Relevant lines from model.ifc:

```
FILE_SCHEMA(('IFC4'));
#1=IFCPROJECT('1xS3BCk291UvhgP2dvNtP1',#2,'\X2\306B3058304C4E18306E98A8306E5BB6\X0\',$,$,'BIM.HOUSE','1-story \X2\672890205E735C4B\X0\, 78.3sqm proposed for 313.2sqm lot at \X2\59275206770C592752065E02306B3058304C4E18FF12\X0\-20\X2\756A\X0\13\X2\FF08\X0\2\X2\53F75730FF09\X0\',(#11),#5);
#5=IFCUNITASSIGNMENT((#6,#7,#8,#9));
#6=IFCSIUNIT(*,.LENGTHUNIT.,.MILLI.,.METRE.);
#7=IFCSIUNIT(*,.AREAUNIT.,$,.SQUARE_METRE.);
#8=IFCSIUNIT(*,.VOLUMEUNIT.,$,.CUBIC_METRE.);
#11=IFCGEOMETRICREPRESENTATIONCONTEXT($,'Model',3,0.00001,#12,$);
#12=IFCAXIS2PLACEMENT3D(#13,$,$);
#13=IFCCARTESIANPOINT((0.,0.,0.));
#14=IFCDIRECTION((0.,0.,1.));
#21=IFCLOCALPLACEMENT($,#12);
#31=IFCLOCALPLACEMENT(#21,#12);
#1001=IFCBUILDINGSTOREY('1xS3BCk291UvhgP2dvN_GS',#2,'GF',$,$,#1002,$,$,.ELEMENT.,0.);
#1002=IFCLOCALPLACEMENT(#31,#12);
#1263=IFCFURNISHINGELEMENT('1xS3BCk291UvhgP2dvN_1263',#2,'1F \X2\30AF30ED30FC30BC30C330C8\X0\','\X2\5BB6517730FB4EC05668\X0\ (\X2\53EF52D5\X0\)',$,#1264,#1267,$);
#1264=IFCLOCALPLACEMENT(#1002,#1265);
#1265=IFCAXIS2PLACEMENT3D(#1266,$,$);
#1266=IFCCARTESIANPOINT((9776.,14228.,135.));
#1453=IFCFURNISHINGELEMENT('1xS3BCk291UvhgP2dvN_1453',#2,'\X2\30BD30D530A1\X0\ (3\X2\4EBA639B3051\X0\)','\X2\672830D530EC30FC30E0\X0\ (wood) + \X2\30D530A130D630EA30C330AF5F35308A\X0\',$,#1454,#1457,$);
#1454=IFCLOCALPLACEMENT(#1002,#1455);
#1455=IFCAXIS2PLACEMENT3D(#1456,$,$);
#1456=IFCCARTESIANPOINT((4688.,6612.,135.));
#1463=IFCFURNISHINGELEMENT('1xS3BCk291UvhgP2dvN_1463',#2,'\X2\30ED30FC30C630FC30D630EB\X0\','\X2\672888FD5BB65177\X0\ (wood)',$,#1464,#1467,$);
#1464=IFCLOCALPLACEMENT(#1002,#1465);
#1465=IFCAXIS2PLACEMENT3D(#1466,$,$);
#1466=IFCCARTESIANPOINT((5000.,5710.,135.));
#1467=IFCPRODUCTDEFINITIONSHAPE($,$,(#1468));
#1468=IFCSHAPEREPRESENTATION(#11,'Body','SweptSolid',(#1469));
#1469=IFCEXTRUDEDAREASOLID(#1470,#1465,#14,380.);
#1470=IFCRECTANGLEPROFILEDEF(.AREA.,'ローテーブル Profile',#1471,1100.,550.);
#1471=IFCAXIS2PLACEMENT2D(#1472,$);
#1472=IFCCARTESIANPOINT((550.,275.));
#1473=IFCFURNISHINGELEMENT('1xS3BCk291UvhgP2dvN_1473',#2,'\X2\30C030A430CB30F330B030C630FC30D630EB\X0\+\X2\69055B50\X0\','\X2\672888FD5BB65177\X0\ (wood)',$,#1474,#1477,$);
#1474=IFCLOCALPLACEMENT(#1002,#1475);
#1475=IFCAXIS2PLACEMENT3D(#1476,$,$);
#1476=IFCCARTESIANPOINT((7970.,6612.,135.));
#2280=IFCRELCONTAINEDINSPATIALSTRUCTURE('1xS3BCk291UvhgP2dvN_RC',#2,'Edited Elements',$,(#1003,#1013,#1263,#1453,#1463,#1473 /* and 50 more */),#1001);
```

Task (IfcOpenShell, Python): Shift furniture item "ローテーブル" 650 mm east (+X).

```python
import ifcopenshell
import ifcopenshell.api.geometry
import ifcopenshell.util.placement

model = ifcopenshell.open("model.ifc")

item = model.by_guid("1xS3BCk291UvhgP2dvN_1463")
matrix = ifcopenshell.util.placement.get_local_placement(item.ObjectPlacement)
matrix[0, 3] += 650.0
ifcopenshell.api.geometry.edit_object_placement(model, product=item, matrix=matrix, is_si=False)

print(ifcopenshell.util.placement.get_local_placement(item.ObjectPlacement).round(3) + 0.0)

model.write("model_rev.ifc")
```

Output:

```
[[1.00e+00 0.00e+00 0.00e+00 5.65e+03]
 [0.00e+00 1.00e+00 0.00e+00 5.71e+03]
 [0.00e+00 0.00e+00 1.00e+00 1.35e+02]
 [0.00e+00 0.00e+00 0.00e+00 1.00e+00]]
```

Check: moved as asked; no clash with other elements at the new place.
